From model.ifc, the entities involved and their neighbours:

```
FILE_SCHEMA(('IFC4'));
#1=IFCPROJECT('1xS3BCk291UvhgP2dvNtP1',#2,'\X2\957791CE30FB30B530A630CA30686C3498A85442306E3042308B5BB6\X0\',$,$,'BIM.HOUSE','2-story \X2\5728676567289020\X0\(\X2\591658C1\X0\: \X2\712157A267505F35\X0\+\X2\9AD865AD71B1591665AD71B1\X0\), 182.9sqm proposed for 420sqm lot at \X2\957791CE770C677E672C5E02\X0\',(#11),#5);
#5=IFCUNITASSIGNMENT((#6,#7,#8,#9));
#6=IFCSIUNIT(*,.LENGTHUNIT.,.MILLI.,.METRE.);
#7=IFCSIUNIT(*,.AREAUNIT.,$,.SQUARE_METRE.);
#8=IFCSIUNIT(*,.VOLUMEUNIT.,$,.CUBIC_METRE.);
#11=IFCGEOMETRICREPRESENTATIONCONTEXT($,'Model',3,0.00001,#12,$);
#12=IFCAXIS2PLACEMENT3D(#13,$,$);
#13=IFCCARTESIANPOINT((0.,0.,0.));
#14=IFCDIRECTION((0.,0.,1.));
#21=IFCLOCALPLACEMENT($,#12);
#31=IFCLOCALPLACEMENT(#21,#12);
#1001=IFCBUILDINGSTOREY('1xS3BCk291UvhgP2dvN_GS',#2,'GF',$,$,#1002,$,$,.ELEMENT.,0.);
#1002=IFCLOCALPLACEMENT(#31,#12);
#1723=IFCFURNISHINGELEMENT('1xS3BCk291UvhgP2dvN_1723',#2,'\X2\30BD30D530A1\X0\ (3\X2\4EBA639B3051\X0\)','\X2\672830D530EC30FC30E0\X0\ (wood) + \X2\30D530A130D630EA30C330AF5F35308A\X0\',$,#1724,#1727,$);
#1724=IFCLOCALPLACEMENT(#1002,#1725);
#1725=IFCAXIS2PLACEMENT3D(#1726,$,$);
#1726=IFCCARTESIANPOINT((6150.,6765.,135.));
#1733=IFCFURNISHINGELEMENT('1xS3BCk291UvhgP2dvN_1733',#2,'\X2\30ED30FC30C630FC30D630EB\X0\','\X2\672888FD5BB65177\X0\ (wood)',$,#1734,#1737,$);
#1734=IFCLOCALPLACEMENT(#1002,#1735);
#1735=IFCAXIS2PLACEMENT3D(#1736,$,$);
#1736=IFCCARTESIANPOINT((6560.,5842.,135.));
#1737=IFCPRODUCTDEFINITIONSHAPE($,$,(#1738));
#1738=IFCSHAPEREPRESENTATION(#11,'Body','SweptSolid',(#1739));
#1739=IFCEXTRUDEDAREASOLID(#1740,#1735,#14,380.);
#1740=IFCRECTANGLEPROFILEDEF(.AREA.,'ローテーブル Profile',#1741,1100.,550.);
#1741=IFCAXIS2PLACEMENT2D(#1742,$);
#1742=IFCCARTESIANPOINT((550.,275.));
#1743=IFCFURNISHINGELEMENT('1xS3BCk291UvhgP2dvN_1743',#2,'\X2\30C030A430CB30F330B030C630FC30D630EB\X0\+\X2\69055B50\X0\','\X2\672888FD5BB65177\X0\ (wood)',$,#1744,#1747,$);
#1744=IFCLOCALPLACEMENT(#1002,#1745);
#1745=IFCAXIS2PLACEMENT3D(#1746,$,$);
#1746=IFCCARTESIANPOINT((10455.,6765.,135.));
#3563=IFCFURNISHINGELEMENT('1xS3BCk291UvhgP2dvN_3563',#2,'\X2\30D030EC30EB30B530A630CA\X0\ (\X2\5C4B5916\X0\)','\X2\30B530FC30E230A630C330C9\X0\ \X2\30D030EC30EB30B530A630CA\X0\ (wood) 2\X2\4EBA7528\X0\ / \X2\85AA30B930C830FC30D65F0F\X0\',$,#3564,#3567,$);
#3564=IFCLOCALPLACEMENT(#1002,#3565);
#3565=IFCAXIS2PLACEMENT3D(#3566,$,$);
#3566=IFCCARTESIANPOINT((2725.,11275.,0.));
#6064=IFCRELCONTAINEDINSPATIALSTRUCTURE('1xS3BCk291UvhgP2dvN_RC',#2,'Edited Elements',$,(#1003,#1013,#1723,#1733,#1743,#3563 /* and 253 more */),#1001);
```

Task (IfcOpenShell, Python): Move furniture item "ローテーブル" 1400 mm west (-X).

```python
import ifcopenshell
import ifcopenshell.api.geometry
import ifcopenshell.util.placement
import ifcopenshell.util.unit

model = ifcopenshell.open("model.ifc")
unit_scale = ifcopenshell.util.unit.calculate_unit_scale(model)

item = model.by_guid("1xS3BCk291UvhgP2dvN_1733")
matrix = ifcopenshell.util.placement.get_local_placement(item.ObjectPlacement)
matrix[0, 3] -= 1.4 / unit_scale
ifcopenshell.api.geometry.edit_object_placement(model, product=item, matrix=matrix, is_si=False)

print(ifcopenshell.util.placement.get_local_placement(item.ObjectPlacement).round(3) + 0.0)

model.write("model_rev.ifc")
```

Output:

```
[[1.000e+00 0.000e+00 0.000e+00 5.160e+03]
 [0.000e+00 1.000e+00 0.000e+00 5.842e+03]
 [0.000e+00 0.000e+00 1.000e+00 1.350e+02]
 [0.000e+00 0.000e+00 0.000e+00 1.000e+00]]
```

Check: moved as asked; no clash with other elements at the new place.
